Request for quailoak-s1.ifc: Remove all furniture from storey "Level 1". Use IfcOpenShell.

First a look at what the model holds.

```python
import ifcopenshell
import ifcopenshell.util.element

model = ifcopenshell.open("quailoak-s1.ifc")
print(model.schema)
storey = next(s for s in model.by_type("IfcBuildingStorey") if s.Name == "Level 1")
furniture = [e for e in ifcopenshell.util.element.get_decomposition(storey) if e.is_a("IfcFurnishingElement")]
seen = {}
for e in furniture:
    element_type = ifcopenshell.util.element.get_type(e)
    name = element_type.Name if element_type not in (None, e) else None
    seen[name] = seen.get(name, 0) + 1
for name, count in sorted(seen.items(), key=str):
    print(count, "x", name)
```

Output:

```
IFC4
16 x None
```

```python
import ifcopenshell
import ifcopenshell.api.root
import ifcopenshell.util.element

model = ifcopenshell.open("quailoak-s1.ifc")

storey = next(s for s in model.by_type("IfcBuildingStorey") if s.Name == "Level 1")
furniture = [e for e in ifcopenshell.util.element.get_decomposition(storey) if e.is_a("IfcFurnishingElement")]

for e in furniture:
    ifcopenshell.api.root.remove_product(model, product=e)
print(len(furniture), "removed")

model.write("quailoak-s1_edited.ifc")
```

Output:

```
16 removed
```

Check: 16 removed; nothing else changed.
